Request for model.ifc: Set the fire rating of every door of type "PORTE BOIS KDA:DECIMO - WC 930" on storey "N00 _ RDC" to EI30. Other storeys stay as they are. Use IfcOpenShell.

First a look at what the model holds.

```python
import ifcopenshell
import ifcopenshell.util.element

model = ifcopenshell.open("model.ifc")
print(model.schema)
storey = next(s for s in model.by_type("IfcBuildingStorey") if s.Name == "N00 _ RDC")
doors = [e for e in ifcopenshell.util.element.get_decomposition(storey) if e.is_a("IfcDoor")]
seen = {}
for e in doors:
    element_type = ifcopenshell.util.element.get_type(e)
    key = (element_type.Name if element_type != e and element_type else None, ifcopenshell.util.element.get_pset(e, "Pset_DoorCommon", "FireRating"))
    seen[key] = seen.get(key, 0) + 1
for (name, value), count in sorted(seen.items(), key=str):
    print(count, "x", name, "|", value)
```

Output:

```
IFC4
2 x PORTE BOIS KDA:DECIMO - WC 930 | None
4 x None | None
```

```python
import ifcopenshell
import ifcopenshell.api.pset
import ifcopenshell.util.element

model = ifcopenshell.open("model.ifc")

storey = next(s for s in model.by_type("IfcBuildingStorey") if s.Name == "N00 _ RDC")
doors = [e for e in ifcopenshell.util.element.get_decomposition(storey) if e.is_a("IfcDoor")]

count = 0
for e in doors:
    element_type = ifcopenshell.util.element.get_type(e)
    if element_type in (None, e) or element_type.Name != "PORTE BOIS KDA:DECIMO - WC 930":
        continue
    # add_pset returns the element's existing set when there is one.
    pset = ifcopenshell.api.pset.add_pset(model, product=e, name="Pset_DoorCommon")
    ifcopenshell.api.pset.edit_pset(model, pset=pset, properties={"FireRating": "EI30"})
    count += 1

print(count, "doors updated")

model.write("model_v2.ifc")
```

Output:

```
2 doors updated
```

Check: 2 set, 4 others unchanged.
